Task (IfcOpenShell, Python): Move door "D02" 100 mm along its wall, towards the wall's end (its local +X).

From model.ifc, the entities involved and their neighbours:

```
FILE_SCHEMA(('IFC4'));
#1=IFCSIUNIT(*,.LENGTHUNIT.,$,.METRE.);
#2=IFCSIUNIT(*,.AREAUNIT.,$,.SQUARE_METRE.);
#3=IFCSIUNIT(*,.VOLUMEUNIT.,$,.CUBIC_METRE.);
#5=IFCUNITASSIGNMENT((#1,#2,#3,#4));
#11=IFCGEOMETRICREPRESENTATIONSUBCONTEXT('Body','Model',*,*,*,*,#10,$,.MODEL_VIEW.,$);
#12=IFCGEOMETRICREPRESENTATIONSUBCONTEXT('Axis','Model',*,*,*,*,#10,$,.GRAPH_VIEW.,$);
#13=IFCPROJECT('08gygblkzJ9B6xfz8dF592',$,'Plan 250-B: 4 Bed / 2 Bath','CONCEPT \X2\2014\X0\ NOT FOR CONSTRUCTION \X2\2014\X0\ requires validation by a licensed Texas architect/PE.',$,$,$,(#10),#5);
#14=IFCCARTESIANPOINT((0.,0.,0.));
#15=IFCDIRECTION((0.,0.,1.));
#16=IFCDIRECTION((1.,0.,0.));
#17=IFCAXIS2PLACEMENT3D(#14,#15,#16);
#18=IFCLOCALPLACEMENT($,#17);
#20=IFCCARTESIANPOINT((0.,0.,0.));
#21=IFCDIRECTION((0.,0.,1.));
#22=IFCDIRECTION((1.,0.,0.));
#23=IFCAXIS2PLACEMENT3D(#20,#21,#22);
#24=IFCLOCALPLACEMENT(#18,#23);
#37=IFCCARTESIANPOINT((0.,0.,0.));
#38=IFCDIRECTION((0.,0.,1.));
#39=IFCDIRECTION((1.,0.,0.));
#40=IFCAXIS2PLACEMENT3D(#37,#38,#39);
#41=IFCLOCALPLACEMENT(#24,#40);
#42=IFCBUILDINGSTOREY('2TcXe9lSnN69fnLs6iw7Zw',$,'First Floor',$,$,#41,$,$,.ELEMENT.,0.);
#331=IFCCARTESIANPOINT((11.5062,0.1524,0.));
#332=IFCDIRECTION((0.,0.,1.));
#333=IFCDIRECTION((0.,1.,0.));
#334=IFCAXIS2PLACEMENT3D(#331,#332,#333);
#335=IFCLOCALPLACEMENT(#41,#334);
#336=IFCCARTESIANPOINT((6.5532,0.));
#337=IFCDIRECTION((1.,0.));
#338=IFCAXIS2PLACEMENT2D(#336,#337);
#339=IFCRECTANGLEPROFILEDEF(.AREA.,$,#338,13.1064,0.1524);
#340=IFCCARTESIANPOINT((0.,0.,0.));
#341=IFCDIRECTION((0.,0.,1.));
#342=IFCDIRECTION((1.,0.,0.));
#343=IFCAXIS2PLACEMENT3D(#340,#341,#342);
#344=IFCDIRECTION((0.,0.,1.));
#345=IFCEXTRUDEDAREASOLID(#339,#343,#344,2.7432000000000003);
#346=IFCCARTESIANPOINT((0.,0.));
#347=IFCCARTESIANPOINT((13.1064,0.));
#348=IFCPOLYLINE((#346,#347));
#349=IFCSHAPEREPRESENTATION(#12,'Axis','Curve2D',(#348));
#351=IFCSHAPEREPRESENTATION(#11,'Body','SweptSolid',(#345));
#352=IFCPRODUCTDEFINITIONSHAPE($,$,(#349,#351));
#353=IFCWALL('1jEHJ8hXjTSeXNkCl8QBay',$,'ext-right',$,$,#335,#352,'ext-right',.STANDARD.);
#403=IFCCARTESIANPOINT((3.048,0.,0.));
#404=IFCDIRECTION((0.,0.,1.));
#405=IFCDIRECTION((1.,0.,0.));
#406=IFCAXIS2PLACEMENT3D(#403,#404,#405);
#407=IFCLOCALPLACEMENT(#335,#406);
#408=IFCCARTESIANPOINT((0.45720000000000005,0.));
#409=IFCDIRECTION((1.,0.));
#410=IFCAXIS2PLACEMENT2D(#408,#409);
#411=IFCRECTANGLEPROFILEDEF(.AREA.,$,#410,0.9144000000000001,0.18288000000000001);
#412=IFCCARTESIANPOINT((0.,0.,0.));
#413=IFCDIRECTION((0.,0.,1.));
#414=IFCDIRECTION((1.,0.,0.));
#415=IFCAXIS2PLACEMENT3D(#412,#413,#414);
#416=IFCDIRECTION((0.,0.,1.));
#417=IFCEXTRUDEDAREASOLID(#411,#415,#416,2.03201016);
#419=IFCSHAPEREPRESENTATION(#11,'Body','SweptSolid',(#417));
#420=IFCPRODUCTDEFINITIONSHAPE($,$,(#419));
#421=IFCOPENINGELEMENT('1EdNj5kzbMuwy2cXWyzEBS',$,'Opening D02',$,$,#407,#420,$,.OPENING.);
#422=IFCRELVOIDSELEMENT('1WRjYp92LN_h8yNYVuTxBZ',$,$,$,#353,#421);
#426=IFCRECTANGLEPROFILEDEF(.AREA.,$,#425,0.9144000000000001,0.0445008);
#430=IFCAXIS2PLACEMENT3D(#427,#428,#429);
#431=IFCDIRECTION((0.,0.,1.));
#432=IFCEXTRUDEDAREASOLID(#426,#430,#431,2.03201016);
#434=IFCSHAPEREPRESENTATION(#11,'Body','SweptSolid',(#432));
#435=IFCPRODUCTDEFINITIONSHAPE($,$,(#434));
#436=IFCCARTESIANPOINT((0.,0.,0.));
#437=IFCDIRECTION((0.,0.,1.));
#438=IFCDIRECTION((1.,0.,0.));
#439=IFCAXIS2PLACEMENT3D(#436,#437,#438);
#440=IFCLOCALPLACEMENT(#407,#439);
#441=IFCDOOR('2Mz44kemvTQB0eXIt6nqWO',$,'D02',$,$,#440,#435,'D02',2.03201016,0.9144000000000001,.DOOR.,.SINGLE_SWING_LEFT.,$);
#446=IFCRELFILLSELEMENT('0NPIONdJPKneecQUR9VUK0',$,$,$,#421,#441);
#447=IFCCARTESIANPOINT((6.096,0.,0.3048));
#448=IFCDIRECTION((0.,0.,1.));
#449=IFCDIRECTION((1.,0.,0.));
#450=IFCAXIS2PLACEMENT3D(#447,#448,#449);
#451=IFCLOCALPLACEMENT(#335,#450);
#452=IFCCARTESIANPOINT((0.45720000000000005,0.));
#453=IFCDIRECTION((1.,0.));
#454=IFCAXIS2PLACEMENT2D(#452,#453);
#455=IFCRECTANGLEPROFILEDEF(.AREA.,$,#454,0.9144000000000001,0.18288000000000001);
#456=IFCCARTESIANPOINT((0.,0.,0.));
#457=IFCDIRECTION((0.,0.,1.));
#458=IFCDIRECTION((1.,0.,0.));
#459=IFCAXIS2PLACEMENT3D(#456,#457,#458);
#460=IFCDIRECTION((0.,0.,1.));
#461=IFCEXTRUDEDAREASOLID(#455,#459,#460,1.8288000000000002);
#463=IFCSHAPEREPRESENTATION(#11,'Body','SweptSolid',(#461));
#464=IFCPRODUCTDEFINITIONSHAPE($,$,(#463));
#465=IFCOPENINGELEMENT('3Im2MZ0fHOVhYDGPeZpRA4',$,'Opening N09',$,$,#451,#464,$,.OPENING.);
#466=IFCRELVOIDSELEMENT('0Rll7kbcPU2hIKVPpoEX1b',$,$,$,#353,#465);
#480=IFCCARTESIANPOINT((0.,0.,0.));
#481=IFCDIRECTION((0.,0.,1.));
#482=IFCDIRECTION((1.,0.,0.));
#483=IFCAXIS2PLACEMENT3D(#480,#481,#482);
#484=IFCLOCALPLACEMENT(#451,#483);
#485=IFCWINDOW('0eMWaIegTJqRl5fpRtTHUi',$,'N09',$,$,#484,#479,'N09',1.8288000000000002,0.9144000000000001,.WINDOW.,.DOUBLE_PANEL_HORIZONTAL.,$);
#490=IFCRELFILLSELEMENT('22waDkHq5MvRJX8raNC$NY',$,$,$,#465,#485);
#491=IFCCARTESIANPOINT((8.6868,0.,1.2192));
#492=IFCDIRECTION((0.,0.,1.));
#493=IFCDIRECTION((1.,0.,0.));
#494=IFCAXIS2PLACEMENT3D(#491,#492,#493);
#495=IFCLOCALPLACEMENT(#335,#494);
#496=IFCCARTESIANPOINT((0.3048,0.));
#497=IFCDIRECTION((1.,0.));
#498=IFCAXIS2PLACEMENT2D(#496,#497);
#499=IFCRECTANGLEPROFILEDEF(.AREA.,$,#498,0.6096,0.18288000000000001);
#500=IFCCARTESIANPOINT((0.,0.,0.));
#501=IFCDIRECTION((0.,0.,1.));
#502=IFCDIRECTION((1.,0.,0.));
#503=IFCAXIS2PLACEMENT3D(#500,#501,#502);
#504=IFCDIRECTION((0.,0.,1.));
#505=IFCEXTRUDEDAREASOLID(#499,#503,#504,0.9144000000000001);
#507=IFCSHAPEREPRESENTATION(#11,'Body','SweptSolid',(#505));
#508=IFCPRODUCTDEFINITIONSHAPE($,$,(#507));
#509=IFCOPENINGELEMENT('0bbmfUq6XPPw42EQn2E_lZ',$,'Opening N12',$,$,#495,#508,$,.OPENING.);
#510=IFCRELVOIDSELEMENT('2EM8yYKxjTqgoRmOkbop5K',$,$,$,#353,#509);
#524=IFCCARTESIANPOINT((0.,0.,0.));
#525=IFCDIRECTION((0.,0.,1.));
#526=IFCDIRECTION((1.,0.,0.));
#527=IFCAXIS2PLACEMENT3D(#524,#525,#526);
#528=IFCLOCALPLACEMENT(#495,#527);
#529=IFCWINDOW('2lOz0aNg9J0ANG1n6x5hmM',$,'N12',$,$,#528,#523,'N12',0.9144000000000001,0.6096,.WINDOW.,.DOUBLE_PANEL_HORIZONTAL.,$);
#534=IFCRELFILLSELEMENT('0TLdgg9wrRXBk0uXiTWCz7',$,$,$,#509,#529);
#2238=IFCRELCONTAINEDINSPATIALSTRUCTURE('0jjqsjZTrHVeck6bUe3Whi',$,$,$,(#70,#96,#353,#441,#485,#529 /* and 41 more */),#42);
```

```python
import ifcopenshell
import ifcopenshell.api.geometry
import ifcopenshell.util.placement
import ifcopenshell.util.unit

model = ifcopenshell.open("model.ifc")
unit_scale = ifcopenshell.util.unit.calculate_unit_scale(model)

door = model.by_id(441)
opening = door.FillsVoids[0].RelatingOpeningElement
wall = opening.VoidsElements[0].RelatingBuildingElement

wall_matrix = ifcopenshell.util.placement.get_local_placement(wall.ObjectPlacement)
shift = wall_matrix[:3, 0] * 0.1 / unit_scale
before = ifcopenshell.util.placement.get_local_placement(door.ObjectPlacement)[:3, 3].copy()

# The door is placed relative to its opening, so it follows when the opening moves.
matrix = ifcopenshell.util.placement.get_local_placement(opening.ObjectPlacement)
matrix[:3, 3] += shift
ifcopenshell.api.geometry.edit_object_placement(
    model, product=opening, matrix=matrix, is_si=False, should_transform_children=True
)

after = ifcopenshell.util.placement.get_local_placement(door.ObjectPlacement)[:3, 3]
print("door moved by", (after - before).round(3) + 0.0)

model.write("model_updated.ifc")
```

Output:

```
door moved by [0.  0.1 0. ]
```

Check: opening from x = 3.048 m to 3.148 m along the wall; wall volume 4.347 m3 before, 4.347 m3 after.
